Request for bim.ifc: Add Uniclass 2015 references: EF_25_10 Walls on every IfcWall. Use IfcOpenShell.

First a look at what the model holds.

```python
import ifcopenshell

model = ifcopenshell.open("bim.ifc")
print(model.schema)
print("classifications:", [c.Name for c in model.by_type("IfcClassification")])
for ifc_class in ("IfcDoor", "IfcRoof", "IfcStair", "IfcWall", "IfcWindow"):
    print(ifc_class, len(model.by_type(ifc_class)))
```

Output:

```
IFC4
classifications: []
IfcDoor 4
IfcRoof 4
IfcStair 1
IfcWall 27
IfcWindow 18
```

```python
import ifcopenshell
import ifcopenshell.api.classification

model = ifcopenshell.open("bim.ifc")

system = ifcopenshell.api.classification.add_classification(model, classification="Uniclass 2015")

codes = {
    "IfcWall": ("EF_25_10", "Walls"),
}
for ifc_class, (code, name) in codes.items():
    products = model.by_type(ifc_class)
    ifcopenshell.api.classification.add_reference(
        model, products=products, classification=system, identification=code, name=name
    )
    print(code, len(products))

model.write("bim_edited.ifc")
```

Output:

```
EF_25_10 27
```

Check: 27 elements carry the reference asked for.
